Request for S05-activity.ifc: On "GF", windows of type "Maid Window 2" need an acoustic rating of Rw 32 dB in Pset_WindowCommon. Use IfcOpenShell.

First a look at what the model holds.

```python
import ifcopenshell
import ifcopenshell.util.element

model = ifcopenshell.open("S05-activity.ifc")
print(model.schema)
storey = next(s for s in model.by_type("IfcBuildingStorey") if s.Name == "GF")
windows = [e for e in ifcopenshell.util.element.get_decomposition(storey) if e.is_a("IfcWindow")]
seen = {}
for e in windows:
    element_type = ifcopenshell.util.element.get_type(e)
    key = (element_type.Name if element_type != e and element_type else None, ifcopenshell.util.element.get_pset(e, "Pset_WindowCommon", "AcousticRating"))
    seen[key] = seen.get(key, 0) + 1
for (name, value), count in sorted(seen.items(), key=str):
    print(count, "x", name, "|", value)
```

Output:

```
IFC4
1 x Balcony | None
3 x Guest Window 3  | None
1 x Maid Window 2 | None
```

```python
import ifcopenshell
import ifcopenshell.api.pset
import ifcopenshell.util.element

model = ifcopenshell.open("S05-activity.ifc")

storey = next(s for s in model.by_type("IfcBuildingStorey") if s.Name == "GF")
windows = [e for e in ifcopenshell.util.element.get_decomposition(storey) if e.is_a("IfcWindow")]

count = 0
for e in windows:
    element_type = ifcopenshell.util.element.get_type(e)
    if element_type in (None, e) or element_type.Name != "Maid Window 2":
        continue
    # add_pset returns the element's existing set when there is one.
    pset = ifcopenshell.api.pset.add_pset(model, product=e, name="Pset_WindowCommon")
    ifcopenshell.api.pset.edit_pset(model, pset=pset, properties={"AcousticRating": "Rw 32 dB"})
    count += 1

print(count, "windows updated")

model.write("S05-activity-out.ifc")
```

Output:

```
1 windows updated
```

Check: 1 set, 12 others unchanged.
